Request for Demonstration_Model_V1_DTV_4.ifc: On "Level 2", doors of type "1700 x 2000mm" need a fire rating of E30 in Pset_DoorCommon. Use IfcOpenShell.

First a look at what the model holds.

```python
import ifcopenshell
import ifcopenshell.util.element

model = ifcopenshell.open("Demonstration_Model_V1_DTV_4.ifc")
print(model.schema)
storey = next(s for s in model.by_type("IfcBuildingStorey") if s.Name == "Level 2")
doors = [e for e in ifcopenshell.util.element.get_decomposition(storey) if e.is_a("IfcDoor")]
seen = {}
for e in doors:
    element_type = ifcopenshell.util.element.get_type(e)
    key = (element_type.Name if element_type != e and element_type else None, ifcopenshell.util.element.get_pset(e, "Pset_DoorCommon", "FireRating"))
    seen[key] = seen.get(key, 0) + 1
for (name, value), count in sorted(seen.items(), key=str):
    print(count, "x", name, "|", value)
```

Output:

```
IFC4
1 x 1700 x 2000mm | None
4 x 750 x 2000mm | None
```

```python
import ifcopenshell
import ifcopenshell.api.pset
import ifcopenshell.util.element

model = ifcopenshell.open("Demonstration_Model_V1_DTV_4.ifc")

storey = next(s for s in model.by_type("IfcBuildingStorey") if s.Name == "Level 2")
doors = [e for e in ifcopenshell.util.element.get_decomposition(storey) if e.is_a("IfcDoor")]

count = 0
for e in doors:
    element_type = ifcopenshell.util.element.get_type(e)
    if element_type in (None, e) or element_type.Name != "1700 x 2000mm":
        continue
    # add_pset returns the element's existing set when there is one.
    pset = ifcopenshell.api.pset.add_pset(model, product=e, name="Pset_DoorCommon")
    ifcopenshell.api.pset.edit_pset(model, pset=pset, properties={"FireRating": "E30"})
    count += 1

print(count, "doors updated")

model.write("Demonstration_Model_V1_DTV_4_edited.ifc")
```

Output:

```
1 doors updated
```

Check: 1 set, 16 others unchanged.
